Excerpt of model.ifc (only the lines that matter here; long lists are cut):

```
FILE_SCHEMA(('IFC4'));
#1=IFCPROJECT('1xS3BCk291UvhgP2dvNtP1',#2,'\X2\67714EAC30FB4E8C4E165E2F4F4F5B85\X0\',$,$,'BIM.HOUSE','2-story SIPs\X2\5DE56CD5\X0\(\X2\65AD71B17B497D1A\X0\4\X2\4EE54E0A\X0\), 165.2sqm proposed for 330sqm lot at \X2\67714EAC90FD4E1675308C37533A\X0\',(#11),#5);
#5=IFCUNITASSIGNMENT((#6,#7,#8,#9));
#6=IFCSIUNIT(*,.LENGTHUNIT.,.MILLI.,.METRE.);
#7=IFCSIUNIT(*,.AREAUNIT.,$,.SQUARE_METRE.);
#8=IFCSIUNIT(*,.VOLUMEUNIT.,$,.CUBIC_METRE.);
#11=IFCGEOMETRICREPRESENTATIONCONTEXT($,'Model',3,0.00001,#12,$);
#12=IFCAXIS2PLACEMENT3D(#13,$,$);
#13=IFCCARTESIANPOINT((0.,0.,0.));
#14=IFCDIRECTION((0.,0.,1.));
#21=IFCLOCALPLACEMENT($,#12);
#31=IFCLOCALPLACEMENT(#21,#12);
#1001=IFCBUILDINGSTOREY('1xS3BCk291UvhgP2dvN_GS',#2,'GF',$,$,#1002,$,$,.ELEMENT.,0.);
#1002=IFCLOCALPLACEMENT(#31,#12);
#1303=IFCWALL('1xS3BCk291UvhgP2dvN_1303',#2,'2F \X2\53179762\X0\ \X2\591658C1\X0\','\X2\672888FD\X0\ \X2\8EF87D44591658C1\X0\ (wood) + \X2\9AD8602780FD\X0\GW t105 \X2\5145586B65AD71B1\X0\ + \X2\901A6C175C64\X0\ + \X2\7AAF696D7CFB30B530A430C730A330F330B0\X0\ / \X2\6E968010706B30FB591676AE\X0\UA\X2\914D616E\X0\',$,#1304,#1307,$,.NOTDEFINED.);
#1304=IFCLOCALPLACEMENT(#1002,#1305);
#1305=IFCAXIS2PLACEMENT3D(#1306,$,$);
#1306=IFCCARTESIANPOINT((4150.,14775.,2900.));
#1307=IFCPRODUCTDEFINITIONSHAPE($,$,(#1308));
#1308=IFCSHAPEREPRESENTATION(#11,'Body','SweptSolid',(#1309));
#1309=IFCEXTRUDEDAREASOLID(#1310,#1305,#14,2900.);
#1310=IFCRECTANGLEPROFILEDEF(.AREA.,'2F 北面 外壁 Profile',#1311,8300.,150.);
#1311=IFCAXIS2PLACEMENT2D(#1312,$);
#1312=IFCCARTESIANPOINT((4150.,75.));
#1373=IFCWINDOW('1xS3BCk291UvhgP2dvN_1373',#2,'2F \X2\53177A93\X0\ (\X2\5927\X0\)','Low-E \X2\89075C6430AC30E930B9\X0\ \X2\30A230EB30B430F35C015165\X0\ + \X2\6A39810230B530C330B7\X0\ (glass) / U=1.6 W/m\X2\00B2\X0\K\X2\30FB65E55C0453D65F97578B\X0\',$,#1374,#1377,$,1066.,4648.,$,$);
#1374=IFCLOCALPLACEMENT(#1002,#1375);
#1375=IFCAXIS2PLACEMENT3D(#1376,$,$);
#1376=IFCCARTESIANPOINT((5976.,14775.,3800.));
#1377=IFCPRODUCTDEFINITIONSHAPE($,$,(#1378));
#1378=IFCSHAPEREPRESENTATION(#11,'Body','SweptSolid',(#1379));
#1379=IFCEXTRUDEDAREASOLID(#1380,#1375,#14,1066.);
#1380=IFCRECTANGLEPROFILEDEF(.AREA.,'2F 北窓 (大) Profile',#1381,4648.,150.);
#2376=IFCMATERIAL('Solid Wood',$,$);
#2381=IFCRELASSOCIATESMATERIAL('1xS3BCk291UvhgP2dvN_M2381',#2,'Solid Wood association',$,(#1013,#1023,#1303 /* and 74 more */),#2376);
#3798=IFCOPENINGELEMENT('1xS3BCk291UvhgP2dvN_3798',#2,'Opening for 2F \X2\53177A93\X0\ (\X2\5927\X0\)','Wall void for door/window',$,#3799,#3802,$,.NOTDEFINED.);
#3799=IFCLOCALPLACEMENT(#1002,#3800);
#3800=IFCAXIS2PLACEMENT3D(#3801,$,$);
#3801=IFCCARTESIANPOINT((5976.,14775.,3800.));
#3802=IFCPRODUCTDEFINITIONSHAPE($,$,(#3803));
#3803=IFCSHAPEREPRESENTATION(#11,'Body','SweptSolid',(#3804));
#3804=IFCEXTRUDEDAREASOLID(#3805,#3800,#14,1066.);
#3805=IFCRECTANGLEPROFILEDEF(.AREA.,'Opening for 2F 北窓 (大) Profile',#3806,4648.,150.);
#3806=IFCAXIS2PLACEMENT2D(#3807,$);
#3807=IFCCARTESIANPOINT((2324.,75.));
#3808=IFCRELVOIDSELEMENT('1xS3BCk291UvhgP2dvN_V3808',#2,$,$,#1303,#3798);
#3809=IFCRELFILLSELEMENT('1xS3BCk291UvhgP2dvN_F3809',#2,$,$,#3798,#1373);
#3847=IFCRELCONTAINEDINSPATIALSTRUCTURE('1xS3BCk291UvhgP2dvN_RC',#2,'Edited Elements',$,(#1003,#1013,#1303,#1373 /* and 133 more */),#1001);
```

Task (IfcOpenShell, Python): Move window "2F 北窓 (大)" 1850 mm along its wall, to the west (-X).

```python
import ifcopenshell
import ifcopenshell.api.geometry
import ifcopenshell.util.placement
import ifcopenshell.util.unit

model = ifcopenshell.open("model.ifc")
unit_scale = ifcopenshell.util.unit.calculate_unit_scale(model)

window = model.by_guid("1xS3BCk291UvhgP2dvN_1373")
opening = window.FillsVoids[0].RelatingOpeningElement
wall = opening.VoidsElements[0].RelatingBuildingElement

wall_matrix = ifcopenshell.util.placement.get_local_placement(wall.ObjectPlacement)
shift = wall_matrix[:3, 0] * -1.85 / unit_scale
before = ifcopenshell.util.placement.get_local_placement(window.ObjectPlacement)[:3, 3].copy()

# The window is not placed relative to its opening, so move both.
for product in (opening, window):
    matrix = ifcopenshell.util.placement.get_local_placement(product.ObjectPlacement)
    matrix[:3, 3] += shift
    ifcopenshell.api.geometry.edit_object_placement(model, product=product, matrix=matrix, is_si=False)

after = ifcopenshell.util.placement.get_local_placement(window.ObjectPlacement)[:3, 3]
print("window moved by", (after - before).round(3) + 0.0)

model.write("model_rev.ifc")
```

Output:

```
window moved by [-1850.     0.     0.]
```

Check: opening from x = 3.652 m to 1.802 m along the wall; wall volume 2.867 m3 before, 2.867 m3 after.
